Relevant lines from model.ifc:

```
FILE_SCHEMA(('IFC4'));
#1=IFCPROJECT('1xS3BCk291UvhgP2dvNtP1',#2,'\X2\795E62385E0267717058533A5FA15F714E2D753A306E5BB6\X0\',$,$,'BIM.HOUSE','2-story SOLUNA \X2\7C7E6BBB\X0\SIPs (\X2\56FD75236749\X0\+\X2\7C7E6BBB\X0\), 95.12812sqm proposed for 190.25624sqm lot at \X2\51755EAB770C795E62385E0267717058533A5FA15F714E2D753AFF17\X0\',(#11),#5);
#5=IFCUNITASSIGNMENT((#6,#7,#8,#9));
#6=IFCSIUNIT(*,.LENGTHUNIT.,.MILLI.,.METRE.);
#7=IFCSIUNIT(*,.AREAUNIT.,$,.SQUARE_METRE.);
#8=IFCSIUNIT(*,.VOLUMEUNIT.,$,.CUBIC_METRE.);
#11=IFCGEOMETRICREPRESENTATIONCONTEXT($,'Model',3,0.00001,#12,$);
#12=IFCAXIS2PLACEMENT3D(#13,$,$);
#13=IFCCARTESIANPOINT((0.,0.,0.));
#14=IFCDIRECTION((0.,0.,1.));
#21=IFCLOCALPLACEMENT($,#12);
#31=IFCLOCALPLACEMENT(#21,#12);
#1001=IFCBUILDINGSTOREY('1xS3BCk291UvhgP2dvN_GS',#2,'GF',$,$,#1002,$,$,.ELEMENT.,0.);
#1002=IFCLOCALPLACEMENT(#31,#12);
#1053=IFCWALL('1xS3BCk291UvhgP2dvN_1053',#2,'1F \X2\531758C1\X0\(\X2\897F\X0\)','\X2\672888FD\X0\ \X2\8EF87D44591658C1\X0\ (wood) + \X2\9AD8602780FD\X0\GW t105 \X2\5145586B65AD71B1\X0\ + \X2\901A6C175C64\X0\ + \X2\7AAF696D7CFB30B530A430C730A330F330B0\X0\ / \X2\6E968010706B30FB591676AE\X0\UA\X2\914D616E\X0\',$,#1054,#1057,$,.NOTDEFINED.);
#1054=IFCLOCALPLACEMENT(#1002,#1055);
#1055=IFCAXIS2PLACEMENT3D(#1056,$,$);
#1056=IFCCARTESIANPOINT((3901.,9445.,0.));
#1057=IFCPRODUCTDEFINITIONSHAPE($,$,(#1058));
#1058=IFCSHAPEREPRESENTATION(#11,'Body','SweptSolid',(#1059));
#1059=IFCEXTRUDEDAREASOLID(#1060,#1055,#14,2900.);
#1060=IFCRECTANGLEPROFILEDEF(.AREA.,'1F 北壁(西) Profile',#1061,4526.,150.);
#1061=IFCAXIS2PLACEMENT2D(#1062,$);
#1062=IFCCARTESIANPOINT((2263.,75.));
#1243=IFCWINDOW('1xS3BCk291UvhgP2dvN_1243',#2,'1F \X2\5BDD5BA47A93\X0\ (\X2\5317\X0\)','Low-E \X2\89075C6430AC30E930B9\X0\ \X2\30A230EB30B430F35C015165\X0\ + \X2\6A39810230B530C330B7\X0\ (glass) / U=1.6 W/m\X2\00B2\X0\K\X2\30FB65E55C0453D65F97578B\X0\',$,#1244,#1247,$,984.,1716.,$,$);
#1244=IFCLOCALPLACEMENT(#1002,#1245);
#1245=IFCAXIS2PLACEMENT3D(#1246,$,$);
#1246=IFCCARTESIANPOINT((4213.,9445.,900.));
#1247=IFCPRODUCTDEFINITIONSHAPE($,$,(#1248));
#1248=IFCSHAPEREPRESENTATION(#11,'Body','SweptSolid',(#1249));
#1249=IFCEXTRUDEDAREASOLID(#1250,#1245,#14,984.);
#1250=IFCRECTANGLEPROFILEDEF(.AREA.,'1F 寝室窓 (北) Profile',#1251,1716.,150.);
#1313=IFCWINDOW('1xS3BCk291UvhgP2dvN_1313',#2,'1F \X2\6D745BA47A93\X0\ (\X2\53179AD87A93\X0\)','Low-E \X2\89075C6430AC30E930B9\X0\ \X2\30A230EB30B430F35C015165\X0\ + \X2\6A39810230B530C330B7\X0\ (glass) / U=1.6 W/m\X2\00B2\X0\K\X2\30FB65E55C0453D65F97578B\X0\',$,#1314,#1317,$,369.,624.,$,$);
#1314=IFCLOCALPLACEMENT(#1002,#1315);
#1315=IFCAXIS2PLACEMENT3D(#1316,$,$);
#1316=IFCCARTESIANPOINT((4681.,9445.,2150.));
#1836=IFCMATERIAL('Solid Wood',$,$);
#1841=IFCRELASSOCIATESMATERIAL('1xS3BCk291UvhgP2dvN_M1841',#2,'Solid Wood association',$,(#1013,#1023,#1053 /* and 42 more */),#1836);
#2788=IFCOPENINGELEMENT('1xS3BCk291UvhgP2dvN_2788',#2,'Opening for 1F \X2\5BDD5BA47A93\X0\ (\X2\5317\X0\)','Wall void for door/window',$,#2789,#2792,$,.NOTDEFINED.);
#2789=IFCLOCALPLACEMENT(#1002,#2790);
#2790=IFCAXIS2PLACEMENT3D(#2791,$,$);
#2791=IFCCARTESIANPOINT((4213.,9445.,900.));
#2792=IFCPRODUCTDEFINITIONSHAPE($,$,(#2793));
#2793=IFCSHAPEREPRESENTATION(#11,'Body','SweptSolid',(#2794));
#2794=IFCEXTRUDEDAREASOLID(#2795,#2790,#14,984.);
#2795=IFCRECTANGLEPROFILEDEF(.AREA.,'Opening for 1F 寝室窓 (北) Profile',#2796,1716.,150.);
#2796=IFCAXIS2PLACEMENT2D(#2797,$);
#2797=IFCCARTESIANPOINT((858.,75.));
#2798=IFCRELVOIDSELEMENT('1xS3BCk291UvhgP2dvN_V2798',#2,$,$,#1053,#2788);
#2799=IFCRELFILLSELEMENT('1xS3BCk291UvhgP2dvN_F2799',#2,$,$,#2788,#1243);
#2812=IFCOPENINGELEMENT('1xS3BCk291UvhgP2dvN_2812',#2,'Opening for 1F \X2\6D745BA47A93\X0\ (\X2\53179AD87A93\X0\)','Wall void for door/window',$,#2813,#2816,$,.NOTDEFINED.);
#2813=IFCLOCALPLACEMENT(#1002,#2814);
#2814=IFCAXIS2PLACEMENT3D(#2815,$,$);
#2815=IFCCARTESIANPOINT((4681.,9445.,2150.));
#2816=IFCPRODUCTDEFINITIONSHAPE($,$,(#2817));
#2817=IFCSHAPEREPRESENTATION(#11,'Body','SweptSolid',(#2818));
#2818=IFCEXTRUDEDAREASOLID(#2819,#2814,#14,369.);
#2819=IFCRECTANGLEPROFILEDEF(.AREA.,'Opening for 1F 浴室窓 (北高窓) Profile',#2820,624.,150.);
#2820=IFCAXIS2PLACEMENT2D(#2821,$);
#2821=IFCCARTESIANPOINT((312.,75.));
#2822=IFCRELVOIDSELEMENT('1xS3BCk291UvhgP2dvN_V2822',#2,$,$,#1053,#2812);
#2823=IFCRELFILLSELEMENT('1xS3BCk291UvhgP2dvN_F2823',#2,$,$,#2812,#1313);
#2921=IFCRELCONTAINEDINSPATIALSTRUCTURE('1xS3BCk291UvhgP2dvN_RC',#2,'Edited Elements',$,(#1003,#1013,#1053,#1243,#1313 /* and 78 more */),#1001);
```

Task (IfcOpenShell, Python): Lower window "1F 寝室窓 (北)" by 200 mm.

```python
import numpy as np
import ifcopenshell
import ifcopenshell.api.geometry
import ifcopenshell.util.placement
import ifcopenshell.util.unit

model = ifcopenshell.open("model.ifc")
unit_scale = ifcopenshell.util.unit.calculate_unit_scale(model)

window = model.by_guid("1xS3BCk291UvhgP2dvN_1243")
opening = window.FillsVoids[0].RelatingOpeningElement
dz = -200.0

shift = np.array([0.0, 0.0, dz])
# The window is not placed relative to its opening, so move both.
for product in (opening, window):
    matrix = ifcopenshell.util.placement.get_local_placement(product.ObjectPlacement)
    matrix[:3, 3] += shift
    ifcopenshell.api.geometry.edit_object_placement(model, product=product, matrix=matrix, is_si=False)

print(f"moved by {dz * unit_scale:+.3f} m")

model.write("model_updated.ifc")
```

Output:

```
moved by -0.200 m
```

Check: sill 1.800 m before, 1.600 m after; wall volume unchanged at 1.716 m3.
